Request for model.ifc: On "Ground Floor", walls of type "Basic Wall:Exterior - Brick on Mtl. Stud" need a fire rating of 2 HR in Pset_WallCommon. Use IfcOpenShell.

First a look at what the model holds.

```python
import ifcopenshell
import ifcopenshell.util.element

model = ifcopenshell.open("model.ifc")
print(model.schema)
storey = next(s for s in model.by_type("IfcBuildingStorey") if s.Name == "Ground Floor")
walls = [e for e in ifcopenshell.util.element.get_decomposition(storey) if e.is_a("IfcWall")]
seen = {}
for e in walls:
    element_type = ifcopenshell.util.element.get_type(e)
    key = (element_type.Name if element_type != e and element_type else None, ifcopenshell.util.element.get_pset(e, "Pset_WallCommon", "FireRating"))
    seen[key] = seen.get(key, 0) + 1
for (name, value), count in sorted(seen.items(), key=str):
    print(count, "x", name, "|", value)
```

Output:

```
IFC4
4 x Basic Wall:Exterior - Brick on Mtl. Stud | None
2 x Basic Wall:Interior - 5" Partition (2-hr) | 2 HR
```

```python
import ifcopenshell
import ifcopenshell.api.pset
import ifcopenshell.util.element

model = ifcopenshell.open("model.ifc")

storey = next(s for s in model.by_type("IfcBuildingStorey") if s.Name == "Ground Floor")
walls = [e for e in ifcopenshell.util.element.get_decomposition(storey) if e.is_a("IfcWall")]

count = 0
for e in walls:
    element_type = ifcopenshell.util.element.get_type(e)
    if element_type in (None, e) or element_type.Name != "Basic Wall:Exterior - Brick on Mtl. Stud":
        continue
    # add_pset returns the element's existing set when there is one.
    pset = ifcopenshell.api.pset.add_pset(model, product=e, name="Pset_WallCommon")
    ifcopenshell.api.pset.edit_pset(model, pset=pset, properties={"FireRating": "2 HR"})
    count += 1

print(count, "walls updated")

model.write("model_rev.ifc")
```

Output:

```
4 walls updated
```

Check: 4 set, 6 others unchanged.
